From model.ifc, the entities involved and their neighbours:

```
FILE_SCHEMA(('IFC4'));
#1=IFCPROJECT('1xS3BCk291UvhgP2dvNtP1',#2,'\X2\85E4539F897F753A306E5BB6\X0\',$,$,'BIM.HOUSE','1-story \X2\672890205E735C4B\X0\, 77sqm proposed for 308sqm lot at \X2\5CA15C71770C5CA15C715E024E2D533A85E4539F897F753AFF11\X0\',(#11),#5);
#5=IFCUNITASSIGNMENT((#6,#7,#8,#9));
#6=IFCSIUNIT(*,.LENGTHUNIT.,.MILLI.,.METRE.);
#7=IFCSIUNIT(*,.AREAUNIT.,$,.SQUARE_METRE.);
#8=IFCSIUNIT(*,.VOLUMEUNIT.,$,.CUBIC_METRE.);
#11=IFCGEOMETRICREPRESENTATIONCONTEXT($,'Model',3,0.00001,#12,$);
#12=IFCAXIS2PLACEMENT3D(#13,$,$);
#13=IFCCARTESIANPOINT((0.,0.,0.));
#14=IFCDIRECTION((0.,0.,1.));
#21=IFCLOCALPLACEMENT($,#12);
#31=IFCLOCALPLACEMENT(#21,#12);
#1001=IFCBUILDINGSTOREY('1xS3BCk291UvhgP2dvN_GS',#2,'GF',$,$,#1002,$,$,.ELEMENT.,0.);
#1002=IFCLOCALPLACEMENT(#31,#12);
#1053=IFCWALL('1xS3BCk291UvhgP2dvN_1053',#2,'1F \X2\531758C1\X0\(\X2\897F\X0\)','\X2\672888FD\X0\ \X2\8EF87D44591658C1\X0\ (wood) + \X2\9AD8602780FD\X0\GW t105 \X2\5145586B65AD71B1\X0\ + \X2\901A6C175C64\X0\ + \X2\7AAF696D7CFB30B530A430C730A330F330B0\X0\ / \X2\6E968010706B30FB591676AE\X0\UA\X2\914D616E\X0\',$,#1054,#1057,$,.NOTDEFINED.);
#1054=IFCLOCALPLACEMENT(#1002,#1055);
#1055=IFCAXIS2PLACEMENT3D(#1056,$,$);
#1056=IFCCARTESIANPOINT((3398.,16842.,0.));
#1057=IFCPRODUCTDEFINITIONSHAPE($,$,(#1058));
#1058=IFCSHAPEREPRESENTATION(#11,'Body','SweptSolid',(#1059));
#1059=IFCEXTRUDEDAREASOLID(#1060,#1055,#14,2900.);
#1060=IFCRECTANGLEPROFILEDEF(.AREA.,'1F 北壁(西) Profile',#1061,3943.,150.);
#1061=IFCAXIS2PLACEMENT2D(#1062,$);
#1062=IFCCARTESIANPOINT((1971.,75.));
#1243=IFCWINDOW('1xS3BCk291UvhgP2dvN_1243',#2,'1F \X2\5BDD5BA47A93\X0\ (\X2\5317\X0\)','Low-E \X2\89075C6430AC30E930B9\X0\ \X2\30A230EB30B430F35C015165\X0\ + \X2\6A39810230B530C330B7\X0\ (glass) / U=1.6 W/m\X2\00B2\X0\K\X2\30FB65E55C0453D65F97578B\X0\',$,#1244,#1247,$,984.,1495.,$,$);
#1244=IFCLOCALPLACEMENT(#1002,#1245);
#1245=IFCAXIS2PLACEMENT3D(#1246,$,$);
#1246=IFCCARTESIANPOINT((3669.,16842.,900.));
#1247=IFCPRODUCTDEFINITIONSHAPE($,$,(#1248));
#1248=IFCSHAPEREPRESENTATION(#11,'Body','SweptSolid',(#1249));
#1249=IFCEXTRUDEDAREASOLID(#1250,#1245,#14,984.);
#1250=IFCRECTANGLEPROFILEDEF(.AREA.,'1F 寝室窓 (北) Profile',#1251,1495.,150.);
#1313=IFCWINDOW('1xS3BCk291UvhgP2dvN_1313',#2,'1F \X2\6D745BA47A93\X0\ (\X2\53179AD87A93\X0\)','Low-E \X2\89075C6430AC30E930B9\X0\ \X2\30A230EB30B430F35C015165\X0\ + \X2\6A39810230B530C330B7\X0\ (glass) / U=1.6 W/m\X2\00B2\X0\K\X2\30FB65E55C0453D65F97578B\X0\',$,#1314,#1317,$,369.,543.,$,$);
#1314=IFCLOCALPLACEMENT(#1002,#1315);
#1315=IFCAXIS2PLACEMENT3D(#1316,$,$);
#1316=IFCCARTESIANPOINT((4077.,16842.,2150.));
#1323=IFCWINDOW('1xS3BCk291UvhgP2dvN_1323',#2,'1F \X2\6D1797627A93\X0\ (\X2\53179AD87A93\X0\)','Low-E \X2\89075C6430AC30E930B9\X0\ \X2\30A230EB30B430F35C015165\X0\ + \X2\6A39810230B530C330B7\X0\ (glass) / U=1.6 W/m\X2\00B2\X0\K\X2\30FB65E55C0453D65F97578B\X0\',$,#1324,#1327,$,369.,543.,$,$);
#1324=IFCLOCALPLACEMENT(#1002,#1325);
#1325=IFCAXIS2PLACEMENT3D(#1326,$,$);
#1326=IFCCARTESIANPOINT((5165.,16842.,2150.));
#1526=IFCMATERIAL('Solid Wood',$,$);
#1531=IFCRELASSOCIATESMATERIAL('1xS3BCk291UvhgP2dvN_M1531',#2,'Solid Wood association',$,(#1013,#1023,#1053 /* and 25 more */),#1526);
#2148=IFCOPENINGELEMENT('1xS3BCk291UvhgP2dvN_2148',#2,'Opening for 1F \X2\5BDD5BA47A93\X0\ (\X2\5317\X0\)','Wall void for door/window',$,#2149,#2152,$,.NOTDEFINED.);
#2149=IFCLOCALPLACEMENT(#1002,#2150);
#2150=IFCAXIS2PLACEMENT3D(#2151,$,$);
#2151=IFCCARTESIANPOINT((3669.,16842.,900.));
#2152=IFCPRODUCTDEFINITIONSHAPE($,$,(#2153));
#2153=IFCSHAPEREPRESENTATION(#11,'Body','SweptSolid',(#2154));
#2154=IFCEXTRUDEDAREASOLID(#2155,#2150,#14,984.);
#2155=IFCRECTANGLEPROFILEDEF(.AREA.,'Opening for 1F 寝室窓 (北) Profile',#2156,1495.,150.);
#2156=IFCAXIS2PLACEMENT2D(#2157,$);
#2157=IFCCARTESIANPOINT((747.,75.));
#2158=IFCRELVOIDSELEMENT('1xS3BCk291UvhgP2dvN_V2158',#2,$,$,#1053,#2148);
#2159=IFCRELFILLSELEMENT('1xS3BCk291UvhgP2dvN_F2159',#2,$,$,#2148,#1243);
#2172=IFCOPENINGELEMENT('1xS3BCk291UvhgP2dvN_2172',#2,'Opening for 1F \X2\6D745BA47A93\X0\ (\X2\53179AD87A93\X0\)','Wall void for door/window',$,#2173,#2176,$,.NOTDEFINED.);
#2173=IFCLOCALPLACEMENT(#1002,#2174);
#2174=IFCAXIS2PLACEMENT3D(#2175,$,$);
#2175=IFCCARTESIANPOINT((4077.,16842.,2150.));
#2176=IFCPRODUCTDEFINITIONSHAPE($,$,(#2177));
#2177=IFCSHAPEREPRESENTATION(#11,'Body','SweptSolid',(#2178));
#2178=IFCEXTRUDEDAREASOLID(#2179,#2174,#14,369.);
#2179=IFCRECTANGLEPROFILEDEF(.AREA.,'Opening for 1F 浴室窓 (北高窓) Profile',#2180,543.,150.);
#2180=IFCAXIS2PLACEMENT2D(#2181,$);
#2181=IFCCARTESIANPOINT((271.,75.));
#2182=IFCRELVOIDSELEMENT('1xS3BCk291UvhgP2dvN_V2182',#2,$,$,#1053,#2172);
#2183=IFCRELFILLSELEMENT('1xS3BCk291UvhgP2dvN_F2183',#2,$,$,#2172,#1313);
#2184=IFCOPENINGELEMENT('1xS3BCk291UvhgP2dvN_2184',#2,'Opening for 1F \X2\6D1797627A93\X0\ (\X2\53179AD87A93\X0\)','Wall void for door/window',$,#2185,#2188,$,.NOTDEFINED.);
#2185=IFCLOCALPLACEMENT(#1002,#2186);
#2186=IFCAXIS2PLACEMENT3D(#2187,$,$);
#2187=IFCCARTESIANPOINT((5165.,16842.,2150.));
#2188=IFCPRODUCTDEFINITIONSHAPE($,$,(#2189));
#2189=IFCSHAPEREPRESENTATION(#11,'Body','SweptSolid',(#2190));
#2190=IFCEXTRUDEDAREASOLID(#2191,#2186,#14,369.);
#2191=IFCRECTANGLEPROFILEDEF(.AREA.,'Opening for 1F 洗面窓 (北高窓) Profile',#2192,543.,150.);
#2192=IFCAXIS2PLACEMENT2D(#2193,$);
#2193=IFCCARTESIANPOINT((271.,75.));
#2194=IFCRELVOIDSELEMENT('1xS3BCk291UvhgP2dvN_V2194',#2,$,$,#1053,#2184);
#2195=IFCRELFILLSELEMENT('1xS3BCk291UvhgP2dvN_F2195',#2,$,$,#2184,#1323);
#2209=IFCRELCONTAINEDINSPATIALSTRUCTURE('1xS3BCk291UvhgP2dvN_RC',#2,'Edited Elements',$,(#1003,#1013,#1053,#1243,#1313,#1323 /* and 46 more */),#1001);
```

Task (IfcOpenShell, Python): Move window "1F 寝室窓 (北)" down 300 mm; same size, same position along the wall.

```python
import numpy as np
import ifcopenshell
import ifcopenshell.api.geometry
import ifcopenshell.util.placement
import ifcopenshell.util.unit

model = ifcopenshell.open("model.ifc")
unit_scale = ifcopenshell.util.unit.calculate_unit_scale(model)

window = model.by_guid("1xS3BCk291UvhgP2dvN_1243")
opening = window.FillsVoids[0].RelatingOpeningElement
dz = -0.3 / unit_scale

shift = np.array([0.0, 0.0, dz])
# The window is not placed relative to its opening, so move both.
for product in (opening, window):
    matrix = ifcopenshell.util.placement.get_local_placement(product.ObjectPlacement)
    matrix[:3, 3] += shift
    ifcopenshell.api.geometry.edit_object_placement(model, product=product, matrix=matrix, is_si=False)

print(f"moved by {dz * unit_scale:+.3f} m")

model.write("model_updated.ifc")
```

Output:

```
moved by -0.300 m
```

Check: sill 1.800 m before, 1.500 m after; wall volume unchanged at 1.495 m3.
